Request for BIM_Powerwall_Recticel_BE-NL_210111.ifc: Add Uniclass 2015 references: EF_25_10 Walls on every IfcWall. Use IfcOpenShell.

First a look at what the model holds.

```python
import ifcopenshell

model = ifcopenshell.open("BIM_Powerwall_Recticel_BE-NL_210111.ifc")
print(model.schema)
print("classifications:", [c.Name for c in model.by_type("IfcClassification")])
for ifc_class in ("IfcDoor", "IfcRoof", "IfcStair", "IfcWall", "IfcWindow"):
    print(ifc_class, len(model.by_type(ifc_class)))
```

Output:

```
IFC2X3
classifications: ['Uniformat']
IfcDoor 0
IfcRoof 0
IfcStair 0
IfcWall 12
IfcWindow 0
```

```python
import ifcopenshell
import ifcopenshell.api.classification

model = ifcopenshell.open("BIM_Powerwall_Recticel_BE-NL_210111.ifc")

# IFC2X3 requires Source and Edition and has no link from the project to the system.
system = model.create_entity("IfcClassification", Source="NBS", Edition="2015", Name="Uniclass 2015")

codes = {
    "IfcWall": ("EF_25_10", "Walls"),
}
for ifc_class, (code, name) in codes.items():
    products = model.by_type(ifc_class)
    ifcopenshell.api.classification.add_reference(
        model, products=products, classification=system, identification=code, name=name
    )
    print(code, len(products))

model.write("BIM_Powerwall_Recticel_BE-NL_210111-out.ifc")
```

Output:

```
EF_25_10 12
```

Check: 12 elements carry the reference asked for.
